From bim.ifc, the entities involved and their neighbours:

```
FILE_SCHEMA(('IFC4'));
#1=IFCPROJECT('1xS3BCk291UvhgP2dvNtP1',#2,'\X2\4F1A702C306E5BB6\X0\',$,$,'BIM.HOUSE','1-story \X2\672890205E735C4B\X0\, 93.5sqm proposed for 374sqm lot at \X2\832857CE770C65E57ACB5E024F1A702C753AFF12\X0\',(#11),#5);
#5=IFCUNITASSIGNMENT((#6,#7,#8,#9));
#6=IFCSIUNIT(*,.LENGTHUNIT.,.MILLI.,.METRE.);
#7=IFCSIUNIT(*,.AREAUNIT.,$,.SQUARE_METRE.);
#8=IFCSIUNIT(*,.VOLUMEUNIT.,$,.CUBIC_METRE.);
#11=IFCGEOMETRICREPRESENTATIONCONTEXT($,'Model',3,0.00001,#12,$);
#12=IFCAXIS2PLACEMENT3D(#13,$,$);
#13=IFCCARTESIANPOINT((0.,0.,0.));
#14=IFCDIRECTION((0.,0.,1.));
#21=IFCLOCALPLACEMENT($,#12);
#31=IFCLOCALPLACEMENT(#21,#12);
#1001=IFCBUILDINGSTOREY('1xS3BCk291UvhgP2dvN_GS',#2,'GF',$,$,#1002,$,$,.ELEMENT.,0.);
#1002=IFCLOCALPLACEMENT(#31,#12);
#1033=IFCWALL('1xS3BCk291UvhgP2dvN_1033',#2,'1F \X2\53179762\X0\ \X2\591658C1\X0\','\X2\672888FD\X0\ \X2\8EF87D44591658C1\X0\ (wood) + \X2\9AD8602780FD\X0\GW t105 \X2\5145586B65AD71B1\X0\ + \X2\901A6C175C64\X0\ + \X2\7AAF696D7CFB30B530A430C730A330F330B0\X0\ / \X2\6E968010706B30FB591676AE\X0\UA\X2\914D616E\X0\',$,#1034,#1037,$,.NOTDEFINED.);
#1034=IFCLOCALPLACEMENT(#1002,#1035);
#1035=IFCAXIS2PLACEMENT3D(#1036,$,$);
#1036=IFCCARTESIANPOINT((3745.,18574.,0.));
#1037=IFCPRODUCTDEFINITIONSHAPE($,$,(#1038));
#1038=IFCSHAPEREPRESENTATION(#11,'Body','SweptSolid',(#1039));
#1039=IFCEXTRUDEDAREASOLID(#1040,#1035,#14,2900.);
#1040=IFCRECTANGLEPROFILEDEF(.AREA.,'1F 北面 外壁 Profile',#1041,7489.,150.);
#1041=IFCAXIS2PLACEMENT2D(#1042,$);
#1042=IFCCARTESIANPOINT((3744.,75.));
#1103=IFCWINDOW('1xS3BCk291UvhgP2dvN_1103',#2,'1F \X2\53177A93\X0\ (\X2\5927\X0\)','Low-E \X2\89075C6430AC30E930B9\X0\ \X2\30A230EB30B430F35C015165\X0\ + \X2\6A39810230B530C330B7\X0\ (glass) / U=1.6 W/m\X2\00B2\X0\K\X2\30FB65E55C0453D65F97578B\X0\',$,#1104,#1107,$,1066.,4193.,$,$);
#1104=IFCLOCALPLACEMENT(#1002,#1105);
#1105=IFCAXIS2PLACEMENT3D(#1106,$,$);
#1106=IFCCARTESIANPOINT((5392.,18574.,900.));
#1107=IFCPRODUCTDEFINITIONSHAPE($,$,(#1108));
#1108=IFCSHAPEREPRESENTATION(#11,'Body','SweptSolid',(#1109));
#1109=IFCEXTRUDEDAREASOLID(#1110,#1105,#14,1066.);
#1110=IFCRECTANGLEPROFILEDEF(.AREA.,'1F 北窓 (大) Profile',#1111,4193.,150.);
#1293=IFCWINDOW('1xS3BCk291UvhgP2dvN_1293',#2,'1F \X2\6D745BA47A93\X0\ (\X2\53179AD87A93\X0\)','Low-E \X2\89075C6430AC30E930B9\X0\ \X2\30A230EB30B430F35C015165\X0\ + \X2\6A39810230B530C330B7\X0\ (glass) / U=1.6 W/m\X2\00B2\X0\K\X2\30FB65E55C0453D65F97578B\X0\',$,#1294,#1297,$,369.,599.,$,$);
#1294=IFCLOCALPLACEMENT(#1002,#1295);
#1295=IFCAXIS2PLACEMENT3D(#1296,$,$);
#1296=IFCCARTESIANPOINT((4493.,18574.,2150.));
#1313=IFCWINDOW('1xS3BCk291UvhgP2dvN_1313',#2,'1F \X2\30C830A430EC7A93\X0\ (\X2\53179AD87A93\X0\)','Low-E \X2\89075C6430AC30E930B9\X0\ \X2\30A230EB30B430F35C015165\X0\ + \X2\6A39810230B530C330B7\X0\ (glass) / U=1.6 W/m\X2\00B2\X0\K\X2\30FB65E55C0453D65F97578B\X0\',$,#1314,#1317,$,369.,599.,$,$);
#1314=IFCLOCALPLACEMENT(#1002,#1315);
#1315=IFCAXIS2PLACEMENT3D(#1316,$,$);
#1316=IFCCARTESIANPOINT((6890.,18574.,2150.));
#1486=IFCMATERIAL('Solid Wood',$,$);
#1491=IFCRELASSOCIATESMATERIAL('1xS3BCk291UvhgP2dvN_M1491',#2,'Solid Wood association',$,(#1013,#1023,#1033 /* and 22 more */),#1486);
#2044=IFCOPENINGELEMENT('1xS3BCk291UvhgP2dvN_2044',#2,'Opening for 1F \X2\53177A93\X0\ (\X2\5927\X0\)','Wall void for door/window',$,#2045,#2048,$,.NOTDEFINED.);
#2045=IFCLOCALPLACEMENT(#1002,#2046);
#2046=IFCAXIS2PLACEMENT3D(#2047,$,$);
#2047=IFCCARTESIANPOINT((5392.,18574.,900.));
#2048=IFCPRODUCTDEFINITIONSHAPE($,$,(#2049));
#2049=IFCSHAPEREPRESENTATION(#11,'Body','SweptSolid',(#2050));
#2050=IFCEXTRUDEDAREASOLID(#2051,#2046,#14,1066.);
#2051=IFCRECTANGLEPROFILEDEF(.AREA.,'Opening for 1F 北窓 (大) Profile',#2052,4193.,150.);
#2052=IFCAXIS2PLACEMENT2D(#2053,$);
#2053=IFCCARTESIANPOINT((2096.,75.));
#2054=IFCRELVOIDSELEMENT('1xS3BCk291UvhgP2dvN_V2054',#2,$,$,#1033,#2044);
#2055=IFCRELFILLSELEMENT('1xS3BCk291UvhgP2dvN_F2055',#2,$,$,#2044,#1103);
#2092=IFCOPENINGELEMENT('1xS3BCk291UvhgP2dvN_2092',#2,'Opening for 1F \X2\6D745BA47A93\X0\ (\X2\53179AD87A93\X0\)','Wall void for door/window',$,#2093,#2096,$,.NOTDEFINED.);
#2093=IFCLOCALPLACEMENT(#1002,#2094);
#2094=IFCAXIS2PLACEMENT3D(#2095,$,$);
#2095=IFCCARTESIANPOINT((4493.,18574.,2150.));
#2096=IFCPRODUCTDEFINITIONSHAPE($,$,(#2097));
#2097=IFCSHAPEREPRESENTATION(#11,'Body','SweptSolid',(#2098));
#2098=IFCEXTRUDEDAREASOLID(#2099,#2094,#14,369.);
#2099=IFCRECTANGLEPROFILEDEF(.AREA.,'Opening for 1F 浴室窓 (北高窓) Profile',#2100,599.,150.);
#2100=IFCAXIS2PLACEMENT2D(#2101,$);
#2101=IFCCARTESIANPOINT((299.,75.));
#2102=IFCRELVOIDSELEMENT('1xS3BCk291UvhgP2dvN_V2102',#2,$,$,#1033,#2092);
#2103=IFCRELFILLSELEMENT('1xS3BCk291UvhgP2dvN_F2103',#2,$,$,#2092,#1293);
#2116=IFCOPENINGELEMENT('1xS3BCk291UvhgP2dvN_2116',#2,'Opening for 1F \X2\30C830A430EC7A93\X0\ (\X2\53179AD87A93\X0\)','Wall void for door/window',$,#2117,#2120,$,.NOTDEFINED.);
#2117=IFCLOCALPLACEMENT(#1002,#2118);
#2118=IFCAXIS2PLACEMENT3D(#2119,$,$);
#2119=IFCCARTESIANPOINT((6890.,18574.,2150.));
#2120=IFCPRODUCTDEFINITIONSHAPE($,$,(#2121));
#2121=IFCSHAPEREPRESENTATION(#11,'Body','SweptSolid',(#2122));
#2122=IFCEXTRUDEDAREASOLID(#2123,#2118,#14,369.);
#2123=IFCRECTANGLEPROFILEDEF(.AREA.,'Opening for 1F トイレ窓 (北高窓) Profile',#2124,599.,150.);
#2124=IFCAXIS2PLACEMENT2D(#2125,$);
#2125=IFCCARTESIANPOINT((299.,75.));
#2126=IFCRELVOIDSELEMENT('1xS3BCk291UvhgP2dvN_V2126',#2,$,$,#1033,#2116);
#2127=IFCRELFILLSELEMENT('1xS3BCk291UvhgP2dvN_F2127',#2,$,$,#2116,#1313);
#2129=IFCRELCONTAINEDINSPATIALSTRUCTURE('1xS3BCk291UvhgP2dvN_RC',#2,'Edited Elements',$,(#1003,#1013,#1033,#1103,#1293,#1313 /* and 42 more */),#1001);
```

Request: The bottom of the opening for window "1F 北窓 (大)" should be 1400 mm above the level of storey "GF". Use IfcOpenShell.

```python
import numpy as np
import ifcopenshell
import ifcopenshell.api.geometry
import ifcopenshell.geom
import ifcopenshell.util.element
import ifcopenshell.util.placement
import ifcopenshell.util.shape
import ifcopenshell.util.unit

model = ifcopenshell.open("bim.ifc")
unit_scale = ifcopenshell.util.unit.calculate_unit_scale(model)

window = model.by_guid("1xS3BCk291UvhgP2dvN_1103")
opening = window.FillsVoids[0].RelatingOpeningElement
storey = ifcopenshell.util.element.get_container(window, ifc_class="IfcBuildingStorey")
level = ifcopenshell.util.placement.get_local_placement(storey.ObjectPlacement)[2, 3]

# The opening's origin need not be at the sill, so measure its lowest point.
shape = ifcopenshell.geom.create_shape(ifcopenshell.geom.settings(), opening)
bottom = ifcopenshell.util.shape.get_shape_bottom_elevation(shape, shape.geometry) / unit_scale
dz = level + 1.4 / unit_scale - bottom

shift = np.array([0.0, 0.0, dz])
# The window is not placed relative to its opening, so move both.
for product in (opening, window):
    matrix = ifcopenshell.util.placement.get_local_placement(product.ObjectPlacement)
    matrix[:3, 3] += shift
    ifcopenshell.api.geometry.edit_object_placement(model, product=product, matrix=matrix, is_si=False)

print(f"moved by {dz * unit_scale:+.3f} m")

model.write("bim_edited.ifc")
```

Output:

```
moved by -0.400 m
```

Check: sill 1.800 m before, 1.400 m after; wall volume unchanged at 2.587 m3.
